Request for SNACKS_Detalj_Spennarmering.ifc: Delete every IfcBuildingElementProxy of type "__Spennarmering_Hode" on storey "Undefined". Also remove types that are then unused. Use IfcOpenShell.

First a look at what the model holds.

```python
import ifcopenshell
import ifcopenshell.util.element

model = ifcopenshell.open("SNACKS_Detalj_Spennarmering.ifc")
print(model.schema)
storey = next(s for s in model.by_type("IfcBuildingStorey") if s.Name == "Undefined")
proxies = [e for e in ifcopenshell.util.element.get_decomposition(storey) if e.is_a("IfcBuildingElementProxy")]
seen = {}
for e in proxies:
    element_type = ifcopenshell.util.element.get_type(e)
    name = element_type.Name if element_type not in (None, e) else None
    seen[name] = seen.get(name, 0) + 1
for name, count in sorted(seen.items(), key=str):
    print(count, "x", name)
```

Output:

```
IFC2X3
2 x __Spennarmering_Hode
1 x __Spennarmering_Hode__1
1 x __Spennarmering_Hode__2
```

```python
import ifcopenshell
import ifcopenshell.api.root
import ifcopenshell.util.element

model = ifcopenshell.open("SNACKS_Detalj_Spennarmering.ifc")

storey = next(s for s in model.by_type("IfcBuildingStorey") if s.Name == "Undefined")
proxies = [e for e in ifcopenshell.util.element.get_decomposition(storey) if e.is_a("IfcBuildingElementProxy")]
targets = [e for e in proxies if (t := ifcopenshell.util.element.get_type(e)) not in (None, e) and t.Name == "__Spennarmering_Hode"]
types = {ifcopenshell.util.element.get_type(e) for e in targets} - {None, *targets}

for e in targets:
    ifcopenshell.api.root.remove_product(model, product=e)
print(len(targets), "removed")

unused = [t for t in types if not ifcopenshell.util.element.get_types(t)]
for t in unused:
    ifcopenshell.api.root.remove_product(model, product=t)
print(len(unused), "unused types removed")

model.write("SNACKS_Detalj_Spennarmering_edited.ifc")
```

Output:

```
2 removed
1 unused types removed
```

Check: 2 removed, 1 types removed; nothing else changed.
